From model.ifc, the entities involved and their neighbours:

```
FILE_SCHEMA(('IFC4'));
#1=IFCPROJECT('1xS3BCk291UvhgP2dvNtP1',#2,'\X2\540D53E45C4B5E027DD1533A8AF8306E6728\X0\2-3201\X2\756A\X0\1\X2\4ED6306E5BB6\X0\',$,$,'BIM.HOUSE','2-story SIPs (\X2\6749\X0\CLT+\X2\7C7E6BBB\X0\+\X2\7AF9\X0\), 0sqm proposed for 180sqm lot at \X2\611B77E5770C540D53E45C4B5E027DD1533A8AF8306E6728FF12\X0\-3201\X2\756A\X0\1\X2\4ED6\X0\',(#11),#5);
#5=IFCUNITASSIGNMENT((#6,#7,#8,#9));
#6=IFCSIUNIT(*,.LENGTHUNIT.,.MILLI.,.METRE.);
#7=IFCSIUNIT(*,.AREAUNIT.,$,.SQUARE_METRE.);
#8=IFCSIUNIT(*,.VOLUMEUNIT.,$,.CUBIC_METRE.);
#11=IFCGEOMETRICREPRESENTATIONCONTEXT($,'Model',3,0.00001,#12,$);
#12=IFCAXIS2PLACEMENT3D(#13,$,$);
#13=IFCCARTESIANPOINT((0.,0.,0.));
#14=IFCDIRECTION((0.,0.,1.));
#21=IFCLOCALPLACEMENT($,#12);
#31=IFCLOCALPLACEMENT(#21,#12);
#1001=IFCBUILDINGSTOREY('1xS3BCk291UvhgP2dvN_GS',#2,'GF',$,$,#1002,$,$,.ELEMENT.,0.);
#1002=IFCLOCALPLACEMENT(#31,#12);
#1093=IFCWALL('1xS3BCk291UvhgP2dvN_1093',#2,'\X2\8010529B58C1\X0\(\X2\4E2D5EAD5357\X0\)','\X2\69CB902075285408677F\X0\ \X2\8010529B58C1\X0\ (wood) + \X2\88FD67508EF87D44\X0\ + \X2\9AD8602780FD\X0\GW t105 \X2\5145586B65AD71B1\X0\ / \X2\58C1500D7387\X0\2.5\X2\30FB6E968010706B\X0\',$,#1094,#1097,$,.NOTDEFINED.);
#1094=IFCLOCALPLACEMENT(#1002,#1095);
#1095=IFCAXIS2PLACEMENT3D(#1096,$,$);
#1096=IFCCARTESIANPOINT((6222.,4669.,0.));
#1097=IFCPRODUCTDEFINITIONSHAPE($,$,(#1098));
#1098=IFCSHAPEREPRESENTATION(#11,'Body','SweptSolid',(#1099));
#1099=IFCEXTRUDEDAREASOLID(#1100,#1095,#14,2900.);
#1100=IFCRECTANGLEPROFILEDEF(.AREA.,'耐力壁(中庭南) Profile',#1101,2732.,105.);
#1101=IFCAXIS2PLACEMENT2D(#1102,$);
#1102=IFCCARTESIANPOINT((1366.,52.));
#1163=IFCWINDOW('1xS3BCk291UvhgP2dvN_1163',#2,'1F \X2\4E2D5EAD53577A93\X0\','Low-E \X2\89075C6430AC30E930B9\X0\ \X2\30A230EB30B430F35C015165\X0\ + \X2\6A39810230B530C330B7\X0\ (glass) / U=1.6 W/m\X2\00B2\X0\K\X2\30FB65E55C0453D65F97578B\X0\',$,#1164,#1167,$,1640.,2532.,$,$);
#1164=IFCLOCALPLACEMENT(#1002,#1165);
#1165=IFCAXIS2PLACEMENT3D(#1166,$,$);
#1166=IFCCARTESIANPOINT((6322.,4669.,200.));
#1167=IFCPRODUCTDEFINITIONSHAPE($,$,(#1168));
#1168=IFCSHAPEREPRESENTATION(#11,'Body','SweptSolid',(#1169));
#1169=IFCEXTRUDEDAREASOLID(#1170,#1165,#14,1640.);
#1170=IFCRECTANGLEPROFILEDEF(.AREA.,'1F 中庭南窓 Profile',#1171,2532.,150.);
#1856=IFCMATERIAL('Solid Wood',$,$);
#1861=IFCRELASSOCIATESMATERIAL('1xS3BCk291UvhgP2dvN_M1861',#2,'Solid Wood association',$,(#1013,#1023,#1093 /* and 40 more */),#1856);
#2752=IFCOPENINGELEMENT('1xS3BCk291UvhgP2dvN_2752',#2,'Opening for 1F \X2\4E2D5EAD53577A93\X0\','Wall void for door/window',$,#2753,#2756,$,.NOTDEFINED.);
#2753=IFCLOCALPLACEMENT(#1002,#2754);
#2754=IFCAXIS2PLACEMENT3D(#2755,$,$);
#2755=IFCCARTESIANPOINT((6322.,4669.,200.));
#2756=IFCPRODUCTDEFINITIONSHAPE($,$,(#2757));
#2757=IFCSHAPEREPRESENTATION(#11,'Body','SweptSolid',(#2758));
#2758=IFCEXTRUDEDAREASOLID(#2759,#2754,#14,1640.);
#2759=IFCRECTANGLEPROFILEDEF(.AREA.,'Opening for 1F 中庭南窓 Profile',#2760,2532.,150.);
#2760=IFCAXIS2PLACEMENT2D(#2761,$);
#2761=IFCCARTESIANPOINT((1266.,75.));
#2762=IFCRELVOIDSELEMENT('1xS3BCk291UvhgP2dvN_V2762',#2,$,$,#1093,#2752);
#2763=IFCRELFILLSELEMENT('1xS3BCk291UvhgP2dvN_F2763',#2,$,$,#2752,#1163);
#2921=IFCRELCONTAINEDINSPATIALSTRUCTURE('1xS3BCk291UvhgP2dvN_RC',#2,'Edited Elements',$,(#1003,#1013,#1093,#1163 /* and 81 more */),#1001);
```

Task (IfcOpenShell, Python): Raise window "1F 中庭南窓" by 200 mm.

```python
import numpy as np
import ifcopenshell
import ifcopenshell.api.geometry
import ifcopenshell.util.placement
import ifcopenshell.util.unit

model = ifcopenshell.open("model.ifc")
unit_scale = ifcopenshell.util.unit.calculate_unit_scale(model)

window = model.by_guid("1xS3BCk291UvhgP2dvN_1163")
opening = window.FillsVoids[0].RelatingOpeningElement
dz = 0.2 / unit_scale

shift = np.array([0.0, 0.0, dz])
# The window is not placed relative to its opening, so move both.
for product in (opening, window):
    matrix = ifcopenshell.util.placement.get_local_placement(product.ObjectPlacement)
    matrix[:3, 3] += shift
    ifcopenshell.api.geometry.edit_object_placement(model, product=product, matrix=matrix, is_si=False)

print(f"moved by {dz * unit_scale:+.3f} m")

model.write("model-out.ifc")
```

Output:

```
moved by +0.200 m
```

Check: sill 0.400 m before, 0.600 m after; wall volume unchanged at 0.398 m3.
